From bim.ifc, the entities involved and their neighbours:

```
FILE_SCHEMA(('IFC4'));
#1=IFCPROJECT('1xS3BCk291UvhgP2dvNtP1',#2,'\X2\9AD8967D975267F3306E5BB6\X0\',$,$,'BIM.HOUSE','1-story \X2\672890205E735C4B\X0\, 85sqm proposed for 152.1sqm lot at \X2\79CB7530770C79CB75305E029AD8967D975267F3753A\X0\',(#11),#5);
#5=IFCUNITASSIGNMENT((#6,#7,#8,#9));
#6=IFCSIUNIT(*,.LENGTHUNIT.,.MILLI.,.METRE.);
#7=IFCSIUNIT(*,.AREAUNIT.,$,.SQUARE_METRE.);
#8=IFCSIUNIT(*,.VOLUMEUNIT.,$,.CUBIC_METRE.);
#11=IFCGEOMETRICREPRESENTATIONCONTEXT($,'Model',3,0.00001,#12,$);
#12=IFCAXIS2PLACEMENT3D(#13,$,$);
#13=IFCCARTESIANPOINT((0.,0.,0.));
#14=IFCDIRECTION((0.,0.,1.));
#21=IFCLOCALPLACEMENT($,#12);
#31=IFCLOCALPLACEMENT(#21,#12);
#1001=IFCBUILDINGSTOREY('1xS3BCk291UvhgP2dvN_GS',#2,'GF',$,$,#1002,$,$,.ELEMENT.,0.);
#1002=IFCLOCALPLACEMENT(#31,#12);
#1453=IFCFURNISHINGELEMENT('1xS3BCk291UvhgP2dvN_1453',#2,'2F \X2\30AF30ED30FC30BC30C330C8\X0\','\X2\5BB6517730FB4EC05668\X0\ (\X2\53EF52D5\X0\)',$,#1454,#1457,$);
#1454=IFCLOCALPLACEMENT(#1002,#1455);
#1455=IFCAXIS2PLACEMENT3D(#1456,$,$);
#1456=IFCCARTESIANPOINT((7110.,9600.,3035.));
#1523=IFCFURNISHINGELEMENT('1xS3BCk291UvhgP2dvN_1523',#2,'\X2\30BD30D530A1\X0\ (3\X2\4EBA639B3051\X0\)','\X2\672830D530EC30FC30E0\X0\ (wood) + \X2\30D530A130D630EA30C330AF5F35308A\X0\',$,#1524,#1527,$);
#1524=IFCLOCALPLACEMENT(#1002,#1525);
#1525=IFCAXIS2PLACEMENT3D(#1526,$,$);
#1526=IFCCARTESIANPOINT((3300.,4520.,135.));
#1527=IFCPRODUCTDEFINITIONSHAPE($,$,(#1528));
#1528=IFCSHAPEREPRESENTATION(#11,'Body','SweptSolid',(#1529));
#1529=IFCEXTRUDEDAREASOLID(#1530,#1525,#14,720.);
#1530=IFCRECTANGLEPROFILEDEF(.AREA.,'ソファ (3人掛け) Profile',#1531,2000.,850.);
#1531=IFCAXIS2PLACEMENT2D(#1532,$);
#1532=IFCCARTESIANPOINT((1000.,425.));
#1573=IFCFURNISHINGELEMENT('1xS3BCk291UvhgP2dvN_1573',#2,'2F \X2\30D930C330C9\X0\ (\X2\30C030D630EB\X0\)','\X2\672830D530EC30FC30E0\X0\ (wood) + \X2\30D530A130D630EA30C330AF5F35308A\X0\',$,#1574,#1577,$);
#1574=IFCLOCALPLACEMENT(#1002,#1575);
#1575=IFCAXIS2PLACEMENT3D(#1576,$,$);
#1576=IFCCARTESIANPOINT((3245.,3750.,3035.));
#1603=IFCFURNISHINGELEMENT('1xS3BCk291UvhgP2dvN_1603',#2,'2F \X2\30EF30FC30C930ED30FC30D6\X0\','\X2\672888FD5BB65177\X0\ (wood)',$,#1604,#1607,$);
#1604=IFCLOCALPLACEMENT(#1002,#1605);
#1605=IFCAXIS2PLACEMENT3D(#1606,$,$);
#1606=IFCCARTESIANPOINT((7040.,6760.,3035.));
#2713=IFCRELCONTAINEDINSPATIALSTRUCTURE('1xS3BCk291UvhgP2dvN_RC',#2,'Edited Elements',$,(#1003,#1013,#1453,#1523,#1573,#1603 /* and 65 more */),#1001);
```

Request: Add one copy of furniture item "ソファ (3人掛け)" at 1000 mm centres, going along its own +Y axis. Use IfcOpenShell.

```python
import ifcopenshell
import ifcopenshell.api.geometry
import ifcopenshell.api.root
import ifcopenshell.util.element
import ifcopenshell.util.placement

model = ifcopenshell.open("bim.ifc")


def reuse_history(source, copy):
    """copy_class also copies each property set's owner history, people and application; keep the originals."""
    for rel in copy.IsDefinedBy:
        if rel.is_a("IfcRelDefinesByProperties") and (history := rel.RelatingPropertyDefinition.OwnerHistory):
            rel.RelatingPropertyDefinition.OwnerHistory = source.OwnerHistory
            ifcopenshell.util.element.remove_deep2(model, history)


source = model.by_guid("1xS3BCk291UvhgP2dvN_1523")
base = ifcopenshell.util.placement.get_local_placement(source.ObjectPlacement)
step = base[:3, 1] * 1000.0

for i in range(1, 2):
    copy = ifcopenshell.api.root.copy_class(model, product=source)
    copy.Representation = ifcopenshell.util.element.copy_deep(
        model, source.Representation, exclude=["IfcGeometricRepresentationContext", "IfcRepresentationMap"]
    )
    reuse_history(source, copy)
    matrix = base.copy()
    matrix[:3, 3] += i * step
    print("added at", matrix[:3, 3].round(3) + 0.0)
    ifcopenshell.api.geometry.edit_object_placement(model, product=copy, matrix=matrix, is_si=False)

model.write("bim_rev.ifc")
```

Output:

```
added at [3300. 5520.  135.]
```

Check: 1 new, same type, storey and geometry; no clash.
